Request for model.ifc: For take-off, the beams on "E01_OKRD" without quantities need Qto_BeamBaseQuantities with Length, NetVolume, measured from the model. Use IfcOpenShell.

First a look at what the model holds.

```python
import ifcopenshell
import ifcopenshell.util.element
import ifcopenshell.util.unit

model = ifcopenshell.open("model.ifc")
print(model.schema)
for unit_type in ("LENGTHUNIT", "AREAUNIT", "VOLUMEUNIT"):
    print(unit_type, ifcopenshell.util.unit.calculate_unit_scale(model, unit_type))
storey = next(s for s in model.by_type("IfcBuildingStorey") if s.Name == "E01_OKRD")
beams = [e for e in ifcopenshell.util.element.get_decomposition(storey) if e.is_a("IfcBeam")]
for e in sorted(beams, key=lambda e: e.id()):
    print(e.id(), e.is_a(), e.Name, list(ifcopenshell.util.element.get_psets(e, qtos_only=True)), sep=" | ")
```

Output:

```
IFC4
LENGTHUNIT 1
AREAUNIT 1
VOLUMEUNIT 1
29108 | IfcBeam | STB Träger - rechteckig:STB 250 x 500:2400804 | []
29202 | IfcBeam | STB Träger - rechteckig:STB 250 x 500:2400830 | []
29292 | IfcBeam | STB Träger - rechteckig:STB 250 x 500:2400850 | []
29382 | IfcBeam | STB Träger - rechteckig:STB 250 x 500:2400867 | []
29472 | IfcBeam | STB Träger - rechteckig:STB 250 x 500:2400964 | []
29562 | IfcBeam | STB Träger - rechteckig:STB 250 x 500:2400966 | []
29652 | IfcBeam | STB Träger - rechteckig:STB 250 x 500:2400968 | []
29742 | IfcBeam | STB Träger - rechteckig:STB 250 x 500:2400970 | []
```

```python
import ifcopenshell
import ifcopenshell.api.pset
import ifcopenshell.geom
import ifcopenshell.util.element
import ifcopenshell.util.shape
import ifcopenshell.util.unit

model = ifcopenshell.open("model.ifc")
unit_scale = ifcopenshell.util.unit.calculate_unit_scale(model)
volume_scale = ifcopenshell.util.unit.calculate_unit_scale(model, "VOLUMEUNIT")
settings = ifcopenshell.geom.settings()

storey = next(s for s in model.by_type("IfcBuildingStorey") if s.Name == "E01_OKRD")
beams = [e for e in ifcopenshell.util.element.get_decomposition(storey) if e.is_a("IfcBeam")]

for e in sorted(beams, key=lambda e: e.id()):
    if ifcopenshell.util.element.get_psets(e, qtos_only=True, should_inherit=False):
        continue
    # Geometry comes back in metres, in the element's own axes.
    shape = ifcopenshell.geom.create_shape(settings, e)
    values = {
        "Length": ifcopenshell.util.shape.get_max_xyz(shape.geometry) / unit_scale,
        "NetVolume": ifcopenshell.util.shape.get_volume(shape.geometry) / volume_scale,
    }
    qto = ifcopenshell.api.pset.add_qto(model, product=e, name="Qto_BeamBaseQuantities")
    ifcopenshell.api.pset.edit_qto(model, qto=qto, properties=values)
    print(e.id(), {k: round(v, 3) for k, v in values.items()})

model.write("model-out.ifc")
```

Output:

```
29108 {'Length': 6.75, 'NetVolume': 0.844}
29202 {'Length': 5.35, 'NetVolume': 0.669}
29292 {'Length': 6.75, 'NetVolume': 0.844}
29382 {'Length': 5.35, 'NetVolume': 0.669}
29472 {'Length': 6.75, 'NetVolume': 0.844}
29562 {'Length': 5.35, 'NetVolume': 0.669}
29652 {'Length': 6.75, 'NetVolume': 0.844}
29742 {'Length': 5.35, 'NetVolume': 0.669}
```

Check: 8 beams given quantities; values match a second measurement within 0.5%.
